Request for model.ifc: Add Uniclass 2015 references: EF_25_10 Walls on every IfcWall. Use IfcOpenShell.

First a look at what the model holds.

```python
import ifcopenshell

model = ifcopenshell.open("model.ifc")
print(model.schema)
print("classifications:", [c.Name for c in model.by_type("IfcClassification")])
for ifc_class in ("IfcDoor", "IfcRoof", "IfcStair", "IfcWall", "IfcWindow"):
    print(ifc_class, len(model.by_type(ifc_class)))
```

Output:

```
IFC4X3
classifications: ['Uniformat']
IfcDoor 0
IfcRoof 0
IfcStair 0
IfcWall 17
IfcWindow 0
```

```python
import ifcopenshell
import ifcopenshell.api.classification

model = ifcopenshell.open("model.ifc")

system = ifcopenshell.api.classification.add_classification(model, classification="Uniclass 2015")

codes = {
    "IfcWall": ("EF_25_10", "Walls"),
}
for ifc_class, (code, name) in codes.items():
    products = model.by_type(ifc_class)
    ifcopenshell.api.classification.add_reference(
        model, products=products, classification=system, identification=code, name=name
    )
    print(code, len(products))

model.write("model_edited.ifc")
```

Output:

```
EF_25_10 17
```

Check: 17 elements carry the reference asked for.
